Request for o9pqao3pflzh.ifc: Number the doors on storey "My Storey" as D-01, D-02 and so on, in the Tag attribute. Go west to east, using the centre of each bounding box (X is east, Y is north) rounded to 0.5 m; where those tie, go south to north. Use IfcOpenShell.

First a look at what the model holds.

```python
import ifcopenshell
import ifcopenshell.util.element
import ifcopenshell.util.placement

model = ifcopenshell.open("o9pqao3pflzh.ifc")
print(model.schema)
storey = next(s for s in model.by_type("IfcBuildingStorey") if s.Name == "My Storey")
doors = [e for e in ifcopenshell.util.element.get_decomposition(storey) if e.is_a("IfcDoor")]
for e in sorted(doors, key=lambda e: e.id()):
    origin = ifcopenshell.util.placement.get_local_placement(e.ObjectPlacement)[:3, 3]
    print(e.id(), e.Tag, e.Name, origin.round(2) + 0.0, sep=" | ")
```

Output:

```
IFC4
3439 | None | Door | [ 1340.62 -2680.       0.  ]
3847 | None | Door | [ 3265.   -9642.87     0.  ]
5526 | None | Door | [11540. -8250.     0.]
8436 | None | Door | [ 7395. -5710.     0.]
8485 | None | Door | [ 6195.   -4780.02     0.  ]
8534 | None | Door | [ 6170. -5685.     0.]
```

```python
import ifcopenshell
import ifcopenshell.geom
import ifcopenshell.util.element
import ifcopenshell.util.shape

model = ifcopenshell.open("o9pqao3pflzh.ifc")
settings = ifcopenshell.geom.settings()
settings.set("use-world-coords", True)


def centre(element):
    shape = ifcopenshell.geom.create_shape(settings, element)
    return ifcopenshell.util.shape.get_bbox_centroid(shape.geometry)


storey = next(s for s in model.by_type("IfcBuildingStorey") if s.Name == "My Storey")
doors = [e for e in ifcopenshell.util.element.get_decomposition(storey) if e.is_a("IfcDoor")]

# Insertion points can sit at a corner or the storey origin, so sort by the geometry (in metres).
centres = {e: centre(e) for e in doors}
doors.sort(key=lambda e: (round(centres[e][0] / 0.5), centres[e][1]))

for i, e in enumerate(doors, start=1):
    number = f"D-{i:02d}"
    e.Tag = number
    print(e.id(), number)

model.write("o9pqao3pflzh_updated.ifc")
```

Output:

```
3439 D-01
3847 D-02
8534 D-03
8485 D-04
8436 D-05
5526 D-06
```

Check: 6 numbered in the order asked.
